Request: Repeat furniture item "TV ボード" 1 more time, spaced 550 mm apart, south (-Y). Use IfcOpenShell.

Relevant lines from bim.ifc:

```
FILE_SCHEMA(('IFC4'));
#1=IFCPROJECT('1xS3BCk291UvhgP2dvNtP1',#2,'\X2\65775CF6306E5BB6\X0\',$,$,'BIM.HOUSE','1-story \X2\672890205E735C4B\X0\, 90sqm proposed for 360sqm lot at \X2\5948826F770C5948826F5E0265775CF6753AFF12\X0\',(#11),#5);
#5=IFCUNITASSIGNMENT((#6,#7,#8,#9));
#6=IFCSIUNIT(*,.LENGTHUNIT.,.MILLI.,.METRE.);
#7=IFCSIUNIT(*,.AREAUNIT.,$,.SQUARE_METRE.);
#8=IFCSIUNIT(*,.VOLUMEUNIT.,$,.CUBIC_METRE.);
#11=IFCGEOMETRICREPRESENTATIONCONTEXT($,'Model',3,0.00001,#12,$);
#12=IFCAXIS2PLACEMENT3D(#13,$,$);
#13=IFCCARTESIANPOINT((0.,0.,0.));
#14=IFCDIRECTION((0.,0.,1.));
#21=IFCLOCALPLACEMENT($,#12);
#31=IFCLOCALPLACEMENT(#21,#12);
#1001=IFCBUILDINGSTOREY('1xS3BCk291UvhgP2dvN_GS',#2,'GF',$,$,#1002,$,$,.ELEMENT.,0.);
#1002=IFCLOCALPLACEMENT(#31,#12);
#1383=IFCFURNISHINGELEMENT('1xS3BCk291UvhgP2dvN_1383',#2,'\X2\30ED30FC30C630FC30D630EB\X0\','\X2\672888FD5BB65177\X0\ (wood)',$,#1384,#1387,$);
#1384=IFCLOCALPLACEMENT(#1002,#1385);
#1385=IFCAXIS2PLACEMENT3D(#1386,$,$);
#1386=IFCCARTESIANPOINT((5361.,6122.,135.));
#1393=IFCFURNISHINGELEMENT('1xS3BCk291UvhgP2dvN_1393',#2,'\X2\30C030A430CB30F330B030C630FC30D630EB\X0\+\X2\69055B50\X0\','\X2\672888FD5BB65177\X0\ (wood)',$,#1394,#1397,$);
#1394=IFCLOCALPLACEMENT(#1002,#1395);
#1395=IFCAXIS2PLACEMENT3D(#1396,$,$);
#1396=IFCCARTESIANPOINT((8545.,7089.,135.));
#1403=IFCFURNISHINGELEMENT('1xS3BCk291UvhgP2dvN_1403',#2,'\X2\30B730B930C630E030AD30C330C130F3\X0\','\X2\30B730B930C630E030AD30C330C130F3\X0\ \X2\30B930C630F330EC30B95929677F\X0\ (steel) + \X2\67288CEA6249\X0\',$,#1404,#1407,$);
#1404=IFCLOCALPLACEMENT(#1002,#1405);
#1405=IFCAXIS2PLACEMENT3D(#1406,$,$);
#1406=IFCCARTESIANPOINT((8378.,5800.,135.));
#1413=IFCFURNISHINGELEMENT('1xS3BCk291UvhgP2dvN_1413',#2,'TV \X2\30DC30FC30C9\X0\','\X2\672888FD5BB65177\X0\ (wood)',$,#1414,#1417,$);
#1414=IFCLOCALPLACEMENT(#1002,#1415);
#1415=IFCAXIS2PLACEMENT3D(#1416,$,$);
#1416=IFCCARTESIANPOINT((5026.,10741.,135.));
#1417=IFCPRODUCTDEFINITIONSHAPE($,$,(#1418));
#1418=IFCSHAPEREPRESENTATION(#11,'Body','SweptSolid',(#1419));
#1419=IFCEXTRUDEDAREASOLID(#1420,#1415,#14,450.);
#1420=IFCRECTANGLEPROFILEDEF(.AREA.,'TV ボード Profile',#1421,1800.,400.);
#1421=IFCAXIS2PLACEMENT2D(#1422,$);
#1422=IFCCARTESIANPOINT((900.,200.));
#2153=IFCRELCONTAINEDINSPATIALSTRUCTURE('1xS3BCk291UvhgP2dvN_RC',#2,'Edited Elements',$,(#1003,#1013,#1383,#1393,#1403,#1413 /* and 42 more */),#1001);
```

```python
import numpy as np
import ifcopenshell
import ifcopenshell.api.geometry
import ifcopenshell.api.root
import ifcopenshell.util.element
import ifcopenshell.util.placement
import ifcopenshell.util.unit

model = ifcopenshell.open("bim.ifc")
unit_scale = ifcopenshell.util.unit.calculate_unit_scale(model)


def reuse_history(source, copy):
    """copy_class also copies each property set's owner history, people and application; keep the originals."""
    for rel in copy.IsDefinedBy:
        if rel.is_a("IfcRelDefinesByProperties") and (history := rel.RelatingPropertyDefinition.OwnerHistory):
            rel.RelatingPropertyDefinition.OwnerHistory = source.OwnerHistory
            ifcopenshell.util.element.remove_deep2(model, history)


source = model.by_guid("1xS3BCk291UvhgP2dvN_1413")
base = ifcopenshell.util.placement.get_local_placement(source.ObjectPlacement)
step = np.array([0.0, -1.0, 0.0]) * 0.55 / unit_scale

for i in range(1, 2):
    copy = ifcopenshell.api.root.copy_class(model, product=source)
    copy.Representation = ifcopenshell.util.element.copy_deep(
        model, source.Representation, exclude=["IfcGeometricRepresentationContext", "IfcRepresentationMap"]
    )
    reuse_history(source, copy)
    matrix = base.copy()
    matrix[:3, 3] += i * step
    print("added at", matrix[:3, 3].round(3) + 0.0)
    ifcopenshell.api.geometry.edit_object_placement(model, product=copy, matrix=matrix, is_si=False)

model.write("bim-out.ifc")
```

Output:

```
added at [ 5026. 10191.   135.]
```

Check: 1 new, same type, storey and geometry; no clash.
